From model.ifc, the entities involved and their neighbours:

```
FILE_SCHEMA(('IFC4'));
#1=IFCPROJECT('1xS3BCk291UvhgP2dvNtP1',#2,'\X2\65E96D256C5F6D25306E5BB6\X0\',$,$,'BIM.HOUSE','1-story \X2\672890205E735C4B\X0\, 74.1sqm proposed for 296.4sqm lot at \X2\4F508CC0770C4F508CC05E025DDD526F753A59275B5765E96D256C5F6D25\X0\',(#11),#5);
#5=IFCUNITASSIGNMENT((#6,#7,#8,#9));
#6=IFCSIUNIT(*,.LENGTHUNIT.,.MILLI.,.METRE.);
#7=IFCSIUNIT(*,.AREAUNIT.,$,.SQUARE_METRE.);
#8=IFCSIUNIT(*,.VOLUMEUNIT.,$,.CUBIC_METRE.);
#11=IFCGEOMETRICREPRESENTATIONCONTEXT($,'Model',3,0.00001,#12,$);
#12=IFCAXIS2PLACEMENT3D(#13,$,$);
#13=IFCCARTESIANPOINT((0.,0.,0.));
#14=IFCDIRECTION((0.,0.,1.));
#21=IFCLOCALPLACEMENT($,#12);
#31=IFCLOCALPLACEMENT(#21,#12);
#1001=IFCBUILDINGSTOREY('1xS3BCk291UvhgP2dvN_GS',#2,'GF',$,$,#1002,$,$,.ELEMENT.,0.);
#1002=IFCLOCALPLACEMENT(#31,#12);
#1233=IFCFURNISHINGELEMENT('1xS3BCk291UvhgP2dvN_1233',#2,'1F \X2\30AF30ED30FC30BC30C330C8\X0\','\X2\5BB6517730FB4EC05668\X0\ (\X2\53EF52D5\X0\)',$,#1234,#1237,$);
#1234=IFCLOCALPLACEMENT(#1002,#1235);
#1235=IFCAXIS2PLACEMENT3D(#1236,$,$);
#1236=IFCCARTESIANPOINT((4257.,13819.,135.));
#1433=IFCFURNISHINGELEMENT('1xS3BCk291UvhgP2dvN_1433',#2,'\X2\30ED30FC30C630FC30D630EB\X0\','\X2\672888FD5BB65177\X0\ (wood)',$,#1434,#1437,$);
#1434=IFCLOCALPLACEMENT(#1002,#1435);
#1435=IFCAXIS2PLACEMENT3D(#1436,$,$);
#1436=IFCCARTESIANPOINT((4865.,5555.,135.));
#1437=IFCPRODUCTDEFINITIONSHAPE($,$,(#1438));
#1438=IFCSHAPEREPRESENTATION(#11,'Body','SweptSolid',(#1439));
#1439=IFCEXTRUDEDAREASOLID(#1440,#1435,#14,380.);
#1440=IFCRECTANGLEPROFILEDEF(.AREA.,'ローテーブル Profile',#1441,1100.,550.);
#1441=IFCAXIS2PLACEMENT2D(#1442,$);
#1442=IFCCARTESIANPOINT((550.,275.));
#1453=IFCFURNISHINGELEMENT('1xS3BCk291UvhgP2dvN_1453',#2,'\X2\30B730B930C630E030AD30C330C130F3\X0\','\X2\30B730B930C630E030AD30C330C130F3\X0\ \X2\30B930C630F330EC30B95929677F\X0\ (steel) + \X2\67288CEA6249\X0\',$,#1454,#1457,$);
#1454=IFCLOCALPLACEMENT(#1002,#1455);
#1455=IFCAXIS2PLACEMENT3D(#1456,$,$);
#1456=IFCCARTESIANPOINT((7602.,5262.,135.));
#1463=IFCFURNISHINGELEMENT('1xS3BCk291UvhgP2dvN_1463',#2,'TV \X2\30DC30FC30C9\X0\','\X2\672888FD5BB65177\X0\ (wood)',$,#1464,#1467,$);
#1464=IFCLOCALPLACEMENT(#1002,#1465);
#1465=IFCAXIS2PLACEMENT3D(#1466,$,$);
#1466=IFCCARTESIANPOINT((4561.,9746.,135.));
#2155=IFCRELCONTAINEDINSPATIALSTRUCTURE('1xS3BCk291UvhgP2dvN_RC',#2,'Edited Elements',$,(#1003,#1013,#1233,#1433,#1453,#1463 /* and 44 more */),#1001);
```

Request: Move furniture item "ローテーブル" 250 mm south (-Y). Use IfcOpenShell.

```python
import ifcopenshell
import ifcopenshell.api.geometry
import ifcopenshell.util.placement

model = ifcopenshell.open("model.ifc")

item = model.by_guid("1xS3BCk291UvhgP2dvN_1433")
matrix = ifcopenshell.util.placement.get_local_placement(item.ObjectPlacement)
matrix[1, 3] -= 250.0
ifcopenshell.api.geometry.edit_object_placement(model, product=item, matrix=matrix, is_si=False)

print(ifcopenshell.util.placement.get_local_placement(item.ObjectPlacement).round(3) + 0.0)

model.write("model_rev.ifc")
```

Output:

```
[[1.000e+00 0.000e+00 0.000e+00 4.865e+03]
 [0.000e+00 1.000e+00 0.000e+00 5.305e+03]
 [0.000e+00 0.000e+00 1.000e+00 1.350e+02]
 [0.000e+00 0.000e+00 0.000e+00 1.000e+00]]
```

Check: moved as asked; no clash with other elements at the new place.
